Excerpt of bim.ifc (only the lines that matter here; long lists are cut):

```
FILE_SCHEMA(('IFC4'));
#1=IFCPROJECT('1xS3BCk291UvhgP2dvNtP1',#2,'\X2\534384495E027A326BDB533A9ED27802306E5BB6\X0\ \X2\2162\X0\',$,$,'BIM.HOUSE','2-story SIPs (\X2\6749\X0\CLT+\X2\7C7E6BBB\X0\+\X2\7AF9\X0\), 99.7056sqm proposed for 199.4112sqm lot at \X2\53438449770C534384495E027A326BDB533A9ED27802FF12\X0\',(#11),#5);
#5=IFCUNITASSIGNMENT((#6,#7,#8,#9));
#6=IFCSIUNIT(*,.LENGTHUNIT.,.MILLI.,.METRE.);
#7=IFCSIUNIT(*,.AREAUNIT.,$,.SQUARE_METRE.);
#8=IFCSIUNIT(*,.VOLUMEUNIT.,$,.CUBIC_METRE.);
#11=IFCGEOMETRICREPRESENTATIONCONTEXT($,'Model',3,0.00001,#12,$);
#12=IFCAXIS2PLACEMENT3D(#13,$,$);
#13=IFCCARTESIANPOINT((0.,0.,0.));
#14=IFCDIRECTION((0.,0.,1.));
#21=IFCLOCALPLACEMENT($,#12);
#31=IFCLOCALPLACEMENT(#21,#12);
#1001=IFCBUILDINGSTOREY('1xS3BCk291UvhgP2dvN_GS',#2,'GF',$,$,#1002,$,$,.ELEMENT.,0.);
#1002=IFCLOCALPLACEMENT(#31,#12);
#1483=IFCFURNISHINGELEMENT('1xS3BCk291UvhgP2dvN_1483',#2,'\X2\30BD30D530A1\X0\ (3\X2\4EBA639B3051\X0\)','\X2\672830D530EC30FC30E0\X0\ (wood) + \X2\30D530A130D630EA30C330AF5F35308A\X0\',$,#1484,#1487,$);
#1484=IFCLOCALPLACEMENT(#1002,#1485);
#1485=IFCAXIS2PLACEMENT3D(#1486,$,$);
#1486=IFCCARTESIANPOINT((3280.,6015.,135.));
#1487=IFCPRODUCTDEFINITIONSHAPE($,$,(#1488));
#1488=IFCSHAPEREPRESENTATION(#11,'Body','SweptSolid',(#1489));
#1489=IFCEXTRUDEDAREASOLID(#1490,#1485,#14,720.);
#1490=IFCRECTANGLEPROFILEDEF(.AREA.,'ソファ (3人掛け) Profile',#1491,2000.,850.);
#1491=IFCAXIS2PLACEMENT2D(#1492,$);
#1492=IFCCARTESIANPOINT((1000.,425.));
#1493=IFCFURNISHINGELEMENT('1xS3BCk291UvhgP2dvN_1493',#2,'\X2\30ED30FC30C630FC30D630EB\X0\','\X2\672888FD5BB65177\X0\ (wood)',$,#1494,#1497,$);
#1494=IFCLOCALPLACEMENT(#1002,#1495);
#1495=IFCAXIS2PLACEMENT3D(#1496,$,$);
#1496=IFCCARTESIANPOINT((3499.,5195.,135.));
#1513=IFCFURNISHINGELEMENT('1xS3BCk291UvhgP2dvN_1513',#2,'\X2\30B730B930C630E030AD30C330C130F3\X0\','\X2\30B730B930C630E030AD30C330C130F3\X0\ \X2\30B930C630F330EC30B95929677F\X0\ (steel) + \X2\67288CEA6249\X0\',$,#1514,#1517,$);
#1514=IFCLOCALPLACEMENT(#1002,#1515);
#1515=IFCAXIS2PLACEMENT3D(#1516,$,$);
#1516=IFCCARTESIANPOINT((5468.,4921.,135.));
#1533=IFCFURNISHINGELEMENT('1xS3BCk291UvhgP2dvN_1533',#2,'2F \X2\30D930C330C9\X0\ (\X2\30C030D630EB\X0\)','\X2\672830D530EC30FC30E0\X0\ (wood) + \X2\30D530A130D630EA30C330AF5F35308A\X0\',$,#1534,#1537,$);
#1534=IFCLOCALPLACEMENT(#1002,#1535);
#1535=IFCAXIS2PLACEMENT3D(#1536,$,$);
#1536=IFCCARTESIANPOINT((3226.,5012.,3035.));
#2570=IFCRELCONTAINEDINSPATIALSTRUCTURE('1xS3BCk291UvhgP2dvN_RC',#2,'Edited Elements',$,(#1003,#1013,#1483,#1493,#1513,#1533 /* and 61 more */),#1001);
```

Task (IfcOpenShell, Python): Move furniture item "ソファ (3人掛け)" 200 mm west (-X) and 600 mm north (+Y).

```python
import ifcopenshell
import ifcopenshell.api.geometry
import ifcopenshell.util.placement

model = ifcopenshell.open("bim.ifc")

item = model.by_guid("1xS3BCk291UvhgP2dvN_1483")
matrix = ifcopenshell.util.placement.get_local_placement(item.ObjectPlacement)
matrix[0, 3] -= 200.0
matrix[1, 3] += 600.0
ifcopenshell.api.geometry.edit_object_placement(model, product=item, matrix=matrix, is_si=False)

print(ifcopenshell.util.placement.get_local_placement(item.ObjectPlacement).round(3) + 0.0)

model.write("bim-out.ifc")
```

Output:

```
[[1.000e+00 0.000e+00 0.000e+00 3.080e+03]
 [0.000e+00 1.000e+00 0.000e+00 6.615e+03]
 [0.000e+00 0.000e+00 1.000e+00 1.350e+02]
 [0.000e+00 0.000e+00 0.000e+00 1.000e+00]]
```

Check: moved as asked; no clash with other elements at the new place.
